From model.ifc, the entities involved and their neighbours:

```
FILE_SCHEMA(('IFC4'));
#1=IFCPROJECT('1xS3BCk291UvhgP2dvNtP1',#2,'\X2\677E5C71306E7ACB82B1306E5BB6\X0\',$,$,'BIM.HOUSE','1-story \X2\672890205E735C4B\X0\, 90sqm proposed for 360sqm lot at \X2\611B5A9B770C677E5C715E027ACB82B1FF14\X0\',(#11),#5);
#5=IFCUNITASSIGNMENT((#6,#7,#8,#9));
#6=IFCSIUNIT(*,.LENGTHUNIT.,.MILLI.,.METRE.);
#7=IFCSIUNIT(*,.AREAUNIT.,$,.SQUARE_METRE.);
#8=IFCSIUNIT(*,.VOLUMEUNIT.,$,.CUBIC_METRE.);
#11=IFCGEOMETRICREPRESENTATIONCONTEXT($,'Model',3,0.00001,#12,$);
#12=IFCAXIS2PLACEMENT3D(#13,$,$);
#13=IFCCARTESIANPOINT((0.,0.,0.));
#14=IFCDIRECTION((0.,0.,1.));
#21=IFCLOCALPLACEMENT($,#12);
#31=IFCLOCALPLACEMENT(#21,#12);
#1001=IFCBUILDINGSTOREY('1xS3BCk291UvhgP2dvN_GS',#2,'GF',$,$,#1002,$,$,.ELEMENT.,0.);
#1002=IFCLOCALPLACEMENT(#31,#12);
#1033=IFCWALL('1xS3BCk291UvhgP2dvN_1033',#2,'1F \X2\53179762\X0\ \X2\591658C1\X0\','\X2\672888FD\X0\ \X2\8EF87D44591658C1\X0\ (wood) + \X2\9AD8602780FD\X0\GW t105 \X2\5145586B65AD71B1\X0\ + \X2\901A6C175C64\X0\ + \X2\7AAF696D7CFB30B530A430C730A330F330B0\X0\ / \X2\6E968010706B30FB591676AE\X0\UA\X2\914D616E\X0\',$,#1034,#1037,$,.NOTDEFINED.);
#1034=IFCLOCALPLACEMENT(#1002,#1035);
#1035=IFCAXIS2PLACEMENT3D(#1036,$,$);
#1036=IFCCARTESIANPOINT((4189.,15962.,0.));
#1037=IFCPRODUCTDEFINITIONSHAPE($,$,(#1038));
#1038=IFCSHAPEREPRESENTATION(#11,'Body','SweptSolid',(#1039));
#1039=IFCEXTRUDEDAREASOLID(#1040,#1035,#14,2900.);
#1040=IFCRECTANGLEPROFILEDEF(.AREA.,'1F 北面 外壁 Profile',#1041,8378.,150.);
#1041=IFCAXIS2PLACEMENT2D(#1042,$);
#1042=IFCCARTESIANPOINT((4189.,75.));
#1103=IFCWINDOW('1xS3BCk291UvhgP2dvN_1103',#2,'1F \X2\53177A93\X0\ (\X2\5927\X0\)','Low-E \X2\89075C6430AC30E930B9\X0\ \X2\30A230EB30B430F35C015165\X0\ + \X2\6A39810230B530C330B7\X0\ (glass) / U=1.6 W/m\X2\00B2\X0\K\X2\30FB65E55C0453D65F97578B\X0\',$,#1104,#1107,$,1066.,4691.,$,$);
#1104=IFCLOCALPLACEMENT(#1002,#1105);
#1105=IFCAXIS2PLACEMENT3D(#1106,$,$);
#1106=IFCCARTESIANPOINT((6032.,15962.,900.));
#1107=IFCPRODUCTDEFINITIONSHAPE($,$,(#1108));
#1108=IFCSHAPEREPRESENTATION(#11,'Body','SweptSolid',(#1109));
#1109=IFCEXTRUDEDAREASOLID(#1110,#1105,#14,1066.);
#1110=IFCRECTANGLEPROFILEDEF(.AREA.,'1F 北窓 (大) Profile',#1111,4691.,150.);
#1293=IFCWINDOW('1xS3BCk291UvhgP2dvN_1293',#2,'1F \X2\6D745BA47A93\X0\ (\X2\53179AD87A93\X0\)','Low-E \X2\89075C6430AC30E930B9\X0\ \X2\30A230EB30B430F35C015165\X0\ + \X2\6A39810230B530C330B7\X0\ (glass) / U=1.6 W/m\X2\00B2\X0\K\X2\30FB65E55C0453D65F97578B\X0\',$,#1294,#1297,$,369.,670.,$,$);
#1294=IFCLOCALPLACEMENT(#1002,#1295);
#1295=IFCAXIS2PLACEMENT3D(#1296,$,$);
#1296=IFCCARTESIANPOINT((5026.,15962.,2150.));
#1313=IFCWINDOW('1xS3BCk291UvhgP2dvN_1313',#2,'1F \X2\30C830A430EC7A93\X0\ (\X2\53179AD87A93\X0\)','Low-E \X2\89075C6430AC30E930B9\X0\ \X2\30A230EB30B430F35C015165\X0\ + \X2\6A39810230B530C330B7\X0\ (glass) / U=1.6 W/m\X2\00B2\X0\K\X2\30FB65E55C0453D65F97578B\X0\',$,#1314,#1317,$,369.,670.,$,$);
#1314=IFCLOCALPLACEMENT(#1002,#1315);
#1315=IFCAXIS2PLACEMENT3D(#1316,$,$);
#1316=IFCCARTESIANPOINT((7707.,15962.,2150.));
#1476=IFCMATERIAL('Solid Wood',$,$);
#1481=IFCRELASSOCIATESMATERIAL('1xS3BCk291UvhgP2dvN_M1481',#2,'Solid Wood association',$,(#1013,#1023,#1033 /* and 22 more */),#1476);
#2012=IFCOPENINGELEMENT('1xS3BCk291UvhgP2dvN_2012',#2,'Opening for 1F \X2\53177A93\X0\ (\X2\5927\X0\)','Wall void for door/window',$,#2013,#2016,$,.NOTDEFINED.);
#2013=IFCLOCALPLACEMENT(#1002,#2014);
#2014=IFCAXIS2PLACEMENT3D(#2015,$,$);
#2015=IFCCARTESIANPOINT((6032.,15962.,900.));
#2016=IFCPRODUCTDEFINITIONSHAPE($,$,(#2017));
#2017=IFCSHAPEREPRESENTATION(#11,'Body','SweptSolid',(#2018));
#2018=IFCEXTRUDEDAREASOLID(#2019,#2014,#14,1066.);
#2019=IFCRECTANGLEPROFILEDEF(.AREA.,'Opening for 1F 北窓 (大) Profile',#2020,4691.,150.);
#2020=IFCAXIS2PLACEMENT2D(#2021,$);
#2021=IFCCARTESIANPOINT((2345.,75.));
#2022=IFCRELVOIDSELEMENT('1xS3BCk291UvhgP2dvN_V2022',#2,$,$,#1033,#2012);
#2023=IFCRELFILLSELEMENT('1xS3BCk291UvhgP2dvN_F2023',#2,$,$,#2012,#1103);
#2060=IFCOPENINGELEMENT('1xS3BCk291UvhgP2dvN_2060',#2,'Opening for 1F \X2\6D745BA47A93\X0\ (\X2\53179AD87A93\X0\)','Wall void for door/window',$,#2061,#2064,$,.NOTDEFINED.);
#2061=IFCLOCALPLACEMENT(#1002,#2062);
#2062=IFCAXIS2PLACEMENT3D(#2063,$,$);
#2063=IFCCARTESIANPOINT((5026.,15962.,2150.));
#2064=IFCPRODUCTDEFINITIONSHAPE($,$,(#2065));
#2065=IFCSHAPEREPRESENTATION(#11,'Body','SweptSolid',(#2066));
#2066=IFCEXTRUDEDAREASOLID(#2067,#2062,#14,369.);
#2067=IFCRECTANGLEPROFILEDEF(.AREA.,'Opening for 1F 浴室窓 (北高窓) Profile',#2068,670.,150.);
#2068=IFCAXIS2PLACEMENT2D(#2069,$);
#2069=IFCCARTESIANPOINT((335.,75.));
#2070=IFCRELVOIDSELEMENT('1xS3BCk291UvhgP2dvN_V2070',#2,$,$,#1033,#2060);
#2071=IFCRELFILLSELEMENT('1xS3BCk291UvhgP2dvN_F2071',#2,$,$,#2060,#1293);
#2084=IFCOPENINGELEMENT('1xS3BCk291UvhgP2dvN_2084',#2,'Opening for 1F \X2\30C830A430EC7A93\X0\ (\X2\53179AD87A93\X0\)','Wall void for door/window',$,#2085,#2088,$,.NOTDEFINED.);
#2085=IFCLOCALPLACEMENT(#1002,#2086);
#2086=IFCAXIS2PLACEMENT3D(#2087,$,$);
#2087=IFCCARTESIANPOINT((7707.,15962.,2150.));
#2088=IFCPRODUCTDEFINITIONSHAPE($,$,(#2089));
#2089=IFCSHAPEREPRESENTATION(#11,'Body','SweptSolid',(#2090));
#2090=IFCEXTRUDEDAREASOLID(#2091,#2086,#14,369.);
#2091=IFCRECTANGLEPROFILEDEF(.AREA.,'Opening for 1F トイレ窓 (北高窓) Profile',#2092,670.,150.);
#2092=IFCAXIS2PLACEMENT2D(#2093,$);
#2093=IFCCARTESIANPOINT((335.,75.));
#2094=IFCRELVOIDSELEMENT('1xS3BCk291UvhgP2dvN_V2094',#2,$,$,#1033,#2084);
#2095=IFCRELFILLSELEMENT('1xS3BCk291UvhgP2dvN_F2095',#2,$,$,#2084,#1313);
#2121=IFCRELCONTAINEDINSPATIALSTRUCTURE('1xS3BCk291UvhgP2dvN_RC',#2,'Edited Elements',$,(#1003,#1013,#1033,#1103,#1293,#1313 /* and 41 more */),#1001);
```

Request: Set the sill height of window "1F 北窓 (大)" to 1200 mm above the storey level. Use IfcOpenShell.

```python
import numpy as np
import ifcopenshell
import ifcopenshell.api.geometry
import ifcopenshell.geom
import ifcopenshell.util.element
import ifcopenshell.util.placement
import ifcopenshell.util.shape
import ifcopenshell.util.unit

model = ifcopenshell.open("model.ifc")
unit_scale = ifcopenshell.util.unit.calculate_unit_scale(model)

window = model.by_guid("1xS3BCk291UvhgP2dvN_1103")
opening = window.FillsVoids[0].RelatingOpeningElement
storey = ifcopenshell.util.element.get_container(window, ifc_class="IfcBuildingStorey")
level = ifcopenshell.util.placement.get_local_placement(storey.ObjectPlacement)[2, 3]

# The opening's origin need not be at the sill, so measure its lowest point.
shape = ifcopenshell.geom.create_shape(ifcopenshell.geom.settings(), opening)
bottom = ifcopenshell.util.shape.get_shape_bottom_elevation(shape, shape.geometry) / unit_scale
dz = level + 1200.0 - bottom

shift = np.array([0.0, 0.0, dz])
# The window is not placed relative to its opening, so move both.
for product in (opening, window):
    matrix = ifcopenshell.util.placement.get_local_placement(product.ObjectPlacement)
    matrix[:3, 3] += shift
    ifcopenshell.api.geometry.edit_object_placement(model, product=product, matrix=matrix, is_si=False)

print(f"moved by {dz * unit_scale:+.3f} m")

model.write("model_updated.ifc")
```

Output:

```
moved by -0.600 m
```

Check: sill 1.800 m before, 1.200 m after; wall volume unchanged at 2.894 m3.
